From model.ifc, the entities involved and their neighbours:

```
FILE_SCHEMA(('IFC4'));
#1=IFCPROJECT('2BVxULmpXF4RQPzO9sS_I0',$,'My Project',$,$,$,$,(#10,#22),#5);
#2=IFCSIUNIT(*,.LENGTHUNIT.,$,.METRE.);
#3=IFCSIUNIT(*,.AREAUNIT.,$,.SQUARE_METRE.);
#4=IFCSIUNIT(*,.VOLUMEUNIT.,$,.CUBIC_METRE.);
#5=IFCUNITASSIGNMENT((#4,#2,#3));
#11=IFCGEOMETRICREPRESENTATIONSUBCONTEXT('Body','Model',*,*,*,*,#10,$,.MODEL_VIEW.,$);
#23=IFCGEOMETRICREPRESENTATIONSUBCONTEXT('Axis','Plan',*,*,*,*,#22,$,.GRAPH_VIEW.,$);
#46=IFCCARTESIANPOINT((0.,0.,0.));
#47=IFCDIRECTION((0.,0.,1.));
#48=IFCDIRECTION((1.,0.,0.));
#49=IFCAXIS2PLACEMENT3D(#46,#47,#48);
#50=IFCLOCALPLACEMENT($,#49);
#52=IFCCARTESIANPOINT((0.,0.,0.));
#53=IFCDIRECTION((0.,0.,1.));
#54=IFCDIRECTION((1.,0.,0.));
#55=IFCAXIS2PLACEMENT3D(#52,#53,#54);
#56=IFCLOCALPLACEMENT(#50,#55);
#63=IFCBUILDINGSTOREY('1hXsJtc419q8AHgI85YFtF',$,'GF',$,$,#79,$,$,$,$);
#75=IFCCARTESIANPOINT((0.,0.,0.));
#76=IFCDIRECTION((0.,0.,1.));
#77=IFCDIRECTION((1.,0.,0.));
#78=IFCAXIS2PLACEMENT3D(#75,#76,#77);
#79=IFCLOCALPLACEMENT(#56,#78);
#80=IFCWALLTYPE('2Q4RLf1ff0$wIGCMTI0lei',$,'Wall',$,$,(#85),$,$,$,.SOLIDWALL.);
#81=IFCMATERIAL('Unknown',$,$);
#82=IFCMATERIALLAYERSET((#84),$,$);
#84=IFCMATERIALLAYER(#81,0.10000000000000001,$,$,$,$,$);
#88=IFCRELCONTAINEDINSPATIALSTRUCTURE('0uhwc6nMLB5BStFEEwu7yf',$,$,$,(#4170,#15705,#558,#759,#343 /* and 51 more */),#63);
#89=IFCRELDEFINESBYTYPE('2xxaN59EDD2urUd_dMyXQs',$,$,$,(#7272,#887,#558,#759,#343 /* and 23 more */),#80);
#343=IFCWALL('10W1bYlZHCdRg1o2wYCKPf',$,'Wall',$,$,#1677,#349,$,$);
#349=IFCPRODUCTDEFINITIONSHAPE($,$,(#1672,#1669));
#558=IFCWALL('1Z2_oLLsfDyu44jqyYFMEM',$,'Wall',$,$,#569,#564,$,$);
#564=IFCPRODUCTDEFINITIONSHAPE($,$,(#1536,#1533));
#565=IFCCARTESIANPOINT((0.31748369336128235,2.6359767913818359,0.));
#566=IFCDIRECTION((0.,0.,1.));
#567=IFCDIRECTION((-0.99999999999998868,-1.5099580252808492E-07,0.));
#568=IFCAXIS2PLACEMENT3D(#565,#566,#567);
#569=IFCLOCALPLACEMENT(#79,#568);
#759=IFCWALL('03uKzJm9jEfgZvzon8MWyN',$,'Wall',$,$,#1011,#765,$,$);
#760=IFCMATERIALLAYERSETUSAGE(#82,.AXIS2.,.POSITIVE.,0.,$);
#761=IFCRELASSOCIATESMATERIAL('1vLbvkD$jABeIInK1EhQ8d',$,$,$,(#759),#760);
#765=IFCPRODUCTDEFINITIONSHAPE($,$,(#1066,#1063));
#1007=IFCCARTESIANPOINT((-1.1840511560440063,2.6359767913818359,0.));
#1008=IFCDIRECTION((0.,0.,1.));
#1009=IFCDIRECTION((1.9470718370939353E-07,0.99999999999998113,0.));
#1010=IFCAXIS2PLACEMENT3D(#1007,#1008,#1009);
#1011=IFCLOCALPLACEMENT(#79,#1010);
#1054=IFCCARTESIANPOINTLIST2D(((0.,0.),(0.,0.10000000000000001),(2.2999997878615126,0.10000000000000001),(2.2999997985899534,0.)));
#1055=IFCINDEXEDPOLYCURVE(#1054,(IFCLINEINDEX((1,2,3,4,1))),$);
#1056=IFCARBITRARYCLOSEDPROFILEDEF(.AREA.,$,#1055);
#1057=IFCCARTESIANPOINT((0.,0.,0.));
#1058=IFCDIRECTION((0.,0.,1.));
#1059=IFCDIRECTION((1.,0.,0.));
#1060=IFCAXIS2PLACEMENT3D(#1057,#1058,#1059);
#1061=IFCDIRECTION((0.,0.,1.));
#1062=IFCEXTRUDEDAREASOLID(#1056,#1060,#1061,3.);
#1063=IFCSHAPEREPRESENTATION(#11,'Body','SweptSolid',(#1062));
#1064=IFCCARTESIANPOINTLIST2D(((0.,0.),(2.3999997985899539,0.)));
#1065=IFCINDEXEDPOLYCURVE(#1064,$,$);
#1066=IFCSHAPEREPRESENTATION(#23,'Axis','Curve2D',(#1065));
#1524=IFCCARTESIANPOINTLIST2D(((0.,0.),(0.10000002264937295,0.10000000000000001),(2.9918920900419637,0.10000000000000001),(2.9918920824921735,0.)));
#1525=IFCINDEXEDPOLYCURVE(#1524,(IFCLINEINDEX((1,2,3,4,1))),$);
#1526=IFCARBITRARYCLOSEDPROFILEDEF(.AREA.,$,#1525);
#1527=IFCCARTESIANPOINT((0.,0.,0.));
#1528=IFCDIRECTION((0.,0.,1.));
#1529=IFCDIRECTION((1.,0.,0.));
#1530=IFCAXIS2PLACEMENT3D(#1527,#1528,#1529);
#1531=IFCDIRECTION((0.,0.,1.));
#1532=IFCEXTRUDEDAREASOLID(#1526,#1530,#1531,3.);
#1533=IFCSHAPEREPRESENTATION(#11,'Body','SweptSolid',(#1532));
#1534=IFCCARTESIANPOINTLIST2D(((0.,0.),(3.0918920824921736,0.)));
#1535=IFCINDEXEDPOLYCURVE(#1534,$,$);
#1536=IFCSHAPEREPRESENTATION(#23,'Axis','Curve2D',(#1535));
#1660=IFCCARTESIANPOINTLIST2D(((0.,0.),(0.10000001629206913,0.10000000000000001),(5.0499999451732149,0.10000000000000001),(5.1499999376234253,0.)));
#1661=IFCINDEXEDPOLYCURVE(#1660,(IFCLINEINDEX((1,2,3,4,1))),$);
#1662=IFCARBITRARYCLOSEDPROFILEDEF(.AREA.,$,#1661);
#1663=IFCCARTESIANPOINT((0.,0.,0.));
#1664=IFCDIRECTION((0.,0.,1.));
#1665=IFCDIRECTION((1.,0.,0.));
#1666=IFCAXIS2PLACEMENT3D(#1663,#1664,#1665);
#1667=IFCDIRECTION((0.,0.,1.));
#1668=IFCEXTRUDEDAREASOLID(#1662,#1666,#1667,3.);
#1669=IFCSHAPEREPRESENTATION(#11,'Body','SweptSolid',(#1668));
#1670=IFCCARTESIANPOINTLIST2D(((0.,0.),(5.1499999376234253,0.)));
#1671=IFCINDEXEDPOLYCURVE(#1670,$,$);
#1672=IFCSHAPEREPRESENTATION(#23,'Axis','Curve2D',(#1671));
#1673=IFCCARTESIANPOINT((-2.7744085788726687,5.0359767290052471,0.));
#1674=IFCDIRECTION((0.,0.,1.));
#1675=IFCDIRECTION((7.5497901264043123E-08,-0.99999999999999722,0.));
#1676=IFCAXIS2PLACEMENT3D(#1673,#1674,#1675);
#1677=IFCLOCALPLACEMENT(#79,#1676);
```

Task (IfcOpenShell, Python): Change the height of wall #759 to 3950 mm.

```python
import ifcopenshell
import ifcopenshell.geom
import ifcopenshell.util.representation
import ifcopenshell.util.shape

model = ifcopenshell.open("model.ifc")
settings = ifcopenshell.geom.settings()


def volume(element):
    """Net volume in cubic metres, openings subtracted."""
    shape = ifcopenshell.geom.create_shape(settings, element)
    return ifcopenshell.util.shape.get_volume(shape.geometry)


wall = model.by_guid("03uKzJm9jEfgZvzon8MWyN")
before = volume(wall)

body = ifcopenshell.util.representation.get_representation(wall, "Model", "Body")
solid = body.Items[0]
old_height = solid.Depth
solid.Depth = 3.95
after = volume(wall)

print(f"height {old_height:g} -> {solid.Depth:g}, volume {before:.3f} -> {after:.3f} m3")

model.write("model_v2.ifc")
```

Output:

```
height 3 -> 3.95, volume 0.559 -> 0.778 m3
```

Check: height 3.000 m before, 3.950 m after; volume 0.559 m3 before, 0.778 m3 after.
